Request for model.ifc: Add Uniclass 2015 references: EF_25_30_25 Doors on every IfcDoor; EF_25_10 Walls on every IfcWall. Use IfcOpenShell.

First a look at what the model holds.

```python
import ifcopenshell

model = ifcopenshell.open("model.ifc")
print(model.schema)
print("classifications:", [c.Name for c in model.by_type("IfcClassification")])
for ifc_class in ("IfcDoor", "IfcRoof", "IfcStair", "IfcWall", "IfcWindow"):
    print(ifc_class, len(model.by_type(ifc_class)))
```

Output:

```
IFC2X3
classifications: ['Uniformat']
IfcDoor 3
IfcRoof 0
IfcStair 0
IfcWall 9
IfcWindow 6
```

```python
import ifcopenshell
import ifcopenshell.api.classification

model = ifcopenshell.open("model.ifc")

# IFC2X3 requires Source and Edition and has no link from the project to the system.
system = model.create_entity("IfcClassification", Source="NBS", Edition="2015", Name="Uniclass 2015")

codes = {
    "IfcDoor": ("EF_25_30_25", "Doors"),
    "IfcWall": ("EF_25_10", "Walls"),
}
for ifc_class, (code, name) in codes.items():
    products = model.by_type(ifc_class)
    ifcopenshell.api.classification.add_reference(
        model, products=products, classification=system, identification=code, name=name
    )
    print(code, len(products))

model.write("model-out.ifc")
```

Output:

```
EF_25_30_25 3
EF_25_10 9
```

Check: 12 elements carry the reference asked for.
